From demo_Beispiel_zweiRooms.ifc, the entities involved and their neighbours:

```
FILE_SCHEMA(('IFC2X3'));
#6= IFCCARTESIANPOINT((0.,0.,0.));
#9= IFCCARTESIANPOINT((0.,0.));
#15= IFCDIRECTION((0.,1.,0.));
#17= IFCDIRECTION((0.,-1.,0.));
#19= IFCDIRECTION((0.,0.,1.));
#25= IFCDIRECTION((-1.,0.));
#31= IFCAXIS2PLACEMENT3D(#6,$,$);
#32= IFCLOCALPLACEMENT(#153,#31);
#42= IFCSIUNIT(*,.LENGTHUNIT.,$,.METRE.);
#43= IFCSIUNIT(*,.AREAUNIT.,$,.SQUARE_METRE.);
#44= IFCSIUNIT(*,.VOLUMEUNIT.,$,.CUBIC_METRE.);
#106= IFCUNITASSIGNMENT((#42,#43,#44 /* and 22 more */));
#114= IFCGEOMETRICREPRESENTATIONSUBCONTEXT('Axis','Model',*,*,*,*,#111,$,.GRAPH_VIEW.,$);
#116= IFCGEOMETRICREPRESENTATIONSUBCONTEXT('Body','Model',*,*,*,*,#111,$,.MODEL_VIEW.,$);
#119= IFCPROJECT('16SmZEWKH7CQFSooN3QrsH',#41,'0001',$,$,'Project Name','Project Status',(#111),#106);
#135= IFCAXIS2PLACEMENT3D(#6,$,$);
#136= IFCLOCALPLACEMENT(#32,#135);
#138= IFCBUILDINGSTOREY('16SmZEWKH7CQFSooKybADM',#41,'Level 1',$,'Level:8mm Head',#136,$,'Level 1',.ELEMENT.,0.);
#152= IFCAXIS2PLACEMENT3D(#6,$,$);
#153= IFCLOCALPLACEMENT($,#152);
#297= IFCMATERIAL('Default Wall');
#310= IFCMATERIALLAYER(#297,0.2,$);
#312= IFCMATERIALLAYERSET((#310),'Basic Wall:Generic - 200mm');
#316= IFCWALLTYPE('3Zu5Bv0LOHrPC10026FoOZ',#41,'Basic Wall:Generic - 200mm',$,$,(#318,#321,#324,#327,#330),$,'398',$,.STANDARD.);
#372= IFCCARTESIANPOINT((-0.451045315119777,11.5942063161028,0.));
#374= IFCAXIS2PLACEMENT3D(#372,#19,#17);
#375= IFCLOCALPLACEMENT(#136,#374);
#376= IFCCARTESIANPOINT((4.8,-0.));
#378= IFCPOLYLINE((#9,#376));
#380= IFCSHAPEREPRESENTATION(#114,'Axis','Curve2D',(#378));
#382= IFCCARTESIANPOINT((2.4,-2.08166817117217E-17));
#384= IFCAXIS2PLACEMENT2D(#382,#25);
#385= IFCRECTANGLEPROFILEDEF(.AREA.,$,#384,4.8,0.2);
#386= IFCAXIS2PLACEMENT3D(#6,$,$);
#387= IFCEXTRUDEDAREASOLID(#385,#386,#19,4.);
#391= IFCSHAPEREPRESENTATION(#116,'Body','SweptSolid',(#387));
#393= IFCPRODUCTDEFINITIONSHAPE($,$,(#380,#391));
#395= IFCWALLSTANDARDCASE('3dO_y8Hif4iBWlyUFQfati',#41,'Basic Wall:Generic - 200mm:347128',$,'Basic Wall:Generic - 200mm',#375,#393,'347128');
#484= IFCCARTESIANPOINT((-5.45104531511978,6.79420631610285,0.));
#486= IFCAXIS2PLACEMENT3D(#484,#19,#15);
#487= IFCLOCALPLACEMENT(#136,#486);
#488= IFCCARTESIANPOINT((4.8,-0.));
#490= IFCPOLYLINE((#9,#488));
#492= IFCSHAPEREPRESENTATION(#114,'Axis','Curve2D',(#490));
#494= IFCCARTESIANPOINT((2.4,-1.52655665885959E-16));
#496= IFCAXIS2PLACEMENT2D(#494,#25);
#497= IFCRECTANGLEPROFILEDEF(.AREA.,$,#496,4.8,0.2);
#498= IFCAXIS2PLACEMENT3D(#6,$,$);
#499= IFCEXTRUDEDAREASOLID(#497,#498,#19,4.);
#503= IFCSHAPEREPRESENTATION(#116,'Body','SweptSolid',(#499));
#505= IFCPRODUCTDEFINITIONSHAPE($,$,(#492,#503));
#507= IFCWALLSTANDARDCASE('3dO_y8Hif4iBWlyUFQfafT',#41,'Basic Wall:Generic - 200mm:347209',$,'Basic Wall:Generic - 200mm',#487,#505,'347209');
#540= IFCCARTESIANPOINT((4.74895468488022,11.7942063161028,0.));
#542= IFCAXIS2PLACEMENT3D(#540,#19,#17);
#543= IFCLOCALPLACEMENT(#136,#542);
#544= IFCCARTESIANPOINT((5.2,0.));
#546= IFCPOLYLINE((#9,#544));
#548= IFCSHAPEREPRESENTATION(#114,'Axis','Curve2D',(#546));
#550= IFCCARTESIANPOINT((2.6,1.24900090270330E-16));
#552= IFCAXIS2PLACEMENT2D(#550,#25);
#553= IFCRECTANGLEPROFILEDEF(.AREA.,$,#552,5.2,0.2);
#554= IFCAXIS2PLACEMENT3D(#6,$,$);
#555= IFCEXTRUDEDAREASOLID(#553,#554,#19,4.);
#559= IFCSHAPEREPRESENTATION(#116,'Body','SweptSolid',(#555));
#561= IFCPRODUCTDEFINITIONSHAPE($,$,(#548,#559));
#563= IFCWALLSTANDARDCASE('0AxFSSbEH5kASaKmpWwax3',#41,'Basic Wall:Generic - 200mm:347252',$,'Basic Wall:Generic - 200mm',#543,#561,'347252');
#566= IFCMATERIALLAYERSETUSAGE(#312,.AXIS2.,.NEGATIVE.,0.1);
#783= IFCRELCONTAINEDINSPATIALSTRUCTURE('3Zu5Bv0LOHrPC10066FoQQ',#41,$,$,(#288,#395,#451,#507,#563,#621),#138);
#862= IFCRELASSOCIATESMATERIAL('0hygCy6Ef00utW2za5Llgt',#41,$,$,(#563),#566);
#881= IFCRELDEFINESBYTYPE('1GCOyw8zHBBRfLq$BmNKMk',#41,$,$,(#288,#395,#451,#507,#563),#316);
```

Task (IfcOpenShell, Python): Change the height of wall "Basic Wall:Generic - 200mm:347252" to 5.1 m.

```python
import ifcopenshell
import ifcopenshell.geom
import ifcopenshell.util.representation
import ifcopenshell.util.shape
import ifcopenshell.util.unit

model = ifcopenshell.open("demo_Beispiel_zweiRooms.ifc")
unit_scale = ifcopenshell.util.unit.calculate_unit_scale(model)
settings = ifcopenshell.geom.settings()


def volume(element):
    """Net volume in cubic metres, openings subtracted."""
    shape = ifcopenshell.geom.create_shape(settings, element)
    return ifcopenshell.util.shape.get_volume(shape.geometry)


wall = model.by_guid("0AxFSSbEH5kASaKmpWwax3")
before = volume(wall)

body = ifcopenshell.util.representation.get_representation(wall, "Model", "Body")
solid = body.Items[0]
old_height = solid.Depth
solid.Depth = 5.1 / unit_scale
after = volume(wall)

print(f"height {old_height:g} -> {solid.Depth:g}, volume {before:.3f} -> {after:.3f} m3")

model.write("demo_Beispiel_zweiRooms_edited.ifc")
```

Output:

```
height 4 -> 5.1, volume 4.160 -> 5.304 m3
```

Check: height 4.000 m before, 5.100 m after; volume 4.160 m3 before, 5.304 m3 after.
